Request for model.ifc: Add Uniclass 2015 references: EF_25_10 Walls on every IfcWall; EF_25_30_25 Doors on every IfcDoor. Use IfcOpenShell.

First a look at what the model holds.

```python
import ifcopenshell

model = ifcopenshell.open("model.ifc")
print(model.schema)
print("classifications:", [c.Name for c in model.by_type("IfcClassification")])
for ifc_class in ("IfcDoor", "IfcRoof", "IfcStair", "IfcWall", "IfcWindow"):
    print(ifc_class, len(model.by_type(ifc_class)))
```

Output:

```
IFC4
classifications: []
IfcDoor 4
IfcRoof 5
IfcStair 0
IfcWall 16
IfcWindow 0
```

```python
import ifcopenshell
import ifcopenshell.api.classification

model = ifcopenshell.open("model.ifc")

system = ifcopenshell.api.classification.add_classification(model, classification="Uniclass 2015")

codes = {
    "IfcWall": ("EF_25_10", "Walls"),
    "IfcDoor": ("EF_25_30_25", "Doors"),
}
for ifc_class, (code, name) in codes.items():
    products = model.by_type(ifc_class)
    ifcopenshell.api.classification.add_reference(
        model, products=products, classification=system, identification=code, name=name
    )
    print(code, len(products))

model.write("model_v2.ifc")
```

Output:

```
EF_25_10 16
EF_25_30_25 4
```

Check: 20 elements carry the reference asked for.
